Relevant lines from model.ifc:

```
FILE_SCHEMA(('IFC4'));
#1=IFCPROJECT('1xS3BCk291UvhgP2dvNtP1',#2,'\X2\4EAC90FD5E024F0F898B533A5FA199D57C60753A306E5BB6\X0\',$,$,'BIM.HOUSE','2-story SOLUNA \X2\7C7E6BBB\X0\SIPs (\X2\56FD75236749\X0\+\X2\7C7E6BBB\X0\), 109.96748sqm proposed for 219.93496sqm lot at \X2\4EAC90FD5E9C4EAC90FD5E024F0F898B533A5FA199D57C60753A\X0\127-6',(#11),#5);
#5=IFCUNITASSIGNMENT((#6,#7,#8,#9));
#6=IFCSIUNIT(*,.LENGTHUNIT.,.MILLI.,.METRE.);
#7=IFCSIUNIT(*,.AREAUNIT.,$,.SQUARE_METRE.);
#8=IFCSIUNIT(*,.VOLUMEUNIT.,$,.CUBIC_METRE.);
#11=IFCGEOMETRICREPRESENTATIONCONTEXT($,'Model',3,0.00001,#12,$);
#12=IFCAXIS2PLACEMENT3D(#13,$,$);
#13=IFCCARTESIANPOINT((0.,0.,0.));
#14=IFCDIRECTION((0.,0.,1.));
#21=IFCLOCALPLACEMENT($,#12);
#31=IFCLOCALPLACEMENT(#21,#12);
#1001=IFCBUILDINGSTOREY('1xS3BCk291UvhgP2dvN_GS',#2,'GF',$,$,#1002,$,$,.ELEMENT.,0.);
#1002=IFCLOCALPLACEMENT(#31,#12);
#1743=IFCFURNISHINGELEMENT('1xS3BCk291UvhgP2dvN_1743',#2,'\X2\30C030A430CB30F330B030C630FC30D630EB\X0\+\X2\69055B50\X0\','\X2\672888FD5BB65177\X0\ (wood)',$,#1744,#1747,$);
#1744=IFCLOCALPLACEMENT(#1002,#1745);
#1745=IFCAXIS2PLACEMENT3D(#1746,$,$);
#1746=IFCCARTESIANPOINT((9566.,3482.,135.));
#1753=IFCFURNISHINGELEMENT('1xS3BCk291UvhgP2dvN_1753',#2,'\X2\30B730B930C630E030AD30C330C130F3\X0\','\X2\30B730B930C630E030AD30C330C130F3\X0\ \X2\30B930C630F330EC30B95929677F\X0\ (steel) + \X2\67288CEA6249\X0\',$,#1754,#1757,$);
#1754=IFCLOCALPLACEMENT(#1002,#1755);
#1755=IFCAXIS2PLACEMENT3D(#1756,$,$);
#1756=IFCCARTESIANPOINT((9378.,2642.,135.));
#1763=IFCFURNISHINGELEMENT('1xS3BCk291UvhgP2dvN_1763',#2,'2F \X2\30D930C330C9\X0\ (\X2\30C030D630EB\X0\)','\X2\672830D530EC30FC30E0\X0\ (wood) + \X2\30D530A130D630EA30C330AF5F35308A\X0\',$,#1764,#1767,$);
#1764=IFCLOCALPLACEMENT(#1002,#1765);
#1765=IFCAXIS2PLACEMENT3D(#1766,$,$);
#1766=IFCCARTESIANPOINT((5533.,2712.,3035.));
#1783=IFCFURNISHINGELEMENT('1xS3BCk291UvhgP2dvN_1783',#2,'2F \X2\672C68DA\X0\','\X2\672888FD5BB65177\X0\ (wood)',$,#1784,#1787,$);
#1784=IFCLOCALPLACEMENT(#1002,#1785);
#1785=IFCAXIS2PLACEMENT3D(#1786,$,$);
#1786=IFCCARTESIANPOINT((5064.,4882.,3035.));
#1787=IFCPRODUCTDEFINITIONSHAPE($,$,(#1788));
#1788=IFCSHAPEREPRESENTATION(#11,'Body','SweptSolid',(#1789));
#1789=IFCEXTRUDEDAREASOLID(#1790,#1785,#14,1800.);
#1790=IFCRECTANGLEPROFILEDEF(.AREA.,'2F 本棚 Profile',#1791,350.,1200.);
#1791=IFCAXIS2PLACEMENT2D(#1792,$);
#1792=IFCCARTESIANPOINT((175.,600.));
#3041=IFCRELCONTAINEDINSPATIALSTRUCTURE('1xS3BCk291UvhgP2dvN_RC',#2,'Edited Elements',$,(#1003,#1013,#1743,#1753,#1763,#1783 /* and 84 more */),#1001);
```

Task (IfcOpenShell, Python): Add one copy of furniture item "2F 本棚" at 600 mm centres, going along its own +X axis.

```python
import ifcopenshell
import ifcopenshell.api.geometry
import ifcopenshell.api.root
import ifcopenshell.util.element
import ifcopenshell.util.placement
import ifcopenshell.util.unit

model = ifcopenshell.open("model.ifc")
unit_scale = ifcopenshell.util.unit.calculate_unit_scale(model)


def reuse_history(source, copy):
    """copy_class also copies each property set's owner history, people and application; keep the originals."""
    for rel in copy.IsDefinedBy:
        if rel.is_a("IfcRelDefinesByProperties") and (history := rel.RelatingPropertyDefinition.OwnerHistory):
            rel.RelatingPropertyDefinition.OwnerHistory = source.OwnerHistory
            ifcopenshell.util.element.remove_deep2(model, history)


source = model.by_guid("1xS3BCk291UvhgP2dvN_1783")
base = ifcopenshell.util.placement.get_local_placement(source.ObjectPlacement)
step = base[:3, 0] * 0.6 / unit_scale

for i in range(1, 2):
    copy = ifcopenshell.api.root.copy_class(model, product=source)
    copy.Representation = ifcopenshell.util.element.copy_deep(
        model, source.Representation, exclude=["IfcGeometricRepresentationContext", "IfcRepresentationMap"]
    )
    reuse_history(source, copy)
    matrix = base.copy()
    matrix[:3, 3] += i * step
    print("added at", matrix[:3, 3].round(3) + 0.0)
    ifcopenshell.api.geometry.edit_object_placement(model, product=copy, matrix=matrix, is_si=False)

model.write("model_rev.ifc")
```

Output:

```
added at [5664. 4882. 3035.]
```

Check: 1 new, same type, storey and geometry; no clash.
